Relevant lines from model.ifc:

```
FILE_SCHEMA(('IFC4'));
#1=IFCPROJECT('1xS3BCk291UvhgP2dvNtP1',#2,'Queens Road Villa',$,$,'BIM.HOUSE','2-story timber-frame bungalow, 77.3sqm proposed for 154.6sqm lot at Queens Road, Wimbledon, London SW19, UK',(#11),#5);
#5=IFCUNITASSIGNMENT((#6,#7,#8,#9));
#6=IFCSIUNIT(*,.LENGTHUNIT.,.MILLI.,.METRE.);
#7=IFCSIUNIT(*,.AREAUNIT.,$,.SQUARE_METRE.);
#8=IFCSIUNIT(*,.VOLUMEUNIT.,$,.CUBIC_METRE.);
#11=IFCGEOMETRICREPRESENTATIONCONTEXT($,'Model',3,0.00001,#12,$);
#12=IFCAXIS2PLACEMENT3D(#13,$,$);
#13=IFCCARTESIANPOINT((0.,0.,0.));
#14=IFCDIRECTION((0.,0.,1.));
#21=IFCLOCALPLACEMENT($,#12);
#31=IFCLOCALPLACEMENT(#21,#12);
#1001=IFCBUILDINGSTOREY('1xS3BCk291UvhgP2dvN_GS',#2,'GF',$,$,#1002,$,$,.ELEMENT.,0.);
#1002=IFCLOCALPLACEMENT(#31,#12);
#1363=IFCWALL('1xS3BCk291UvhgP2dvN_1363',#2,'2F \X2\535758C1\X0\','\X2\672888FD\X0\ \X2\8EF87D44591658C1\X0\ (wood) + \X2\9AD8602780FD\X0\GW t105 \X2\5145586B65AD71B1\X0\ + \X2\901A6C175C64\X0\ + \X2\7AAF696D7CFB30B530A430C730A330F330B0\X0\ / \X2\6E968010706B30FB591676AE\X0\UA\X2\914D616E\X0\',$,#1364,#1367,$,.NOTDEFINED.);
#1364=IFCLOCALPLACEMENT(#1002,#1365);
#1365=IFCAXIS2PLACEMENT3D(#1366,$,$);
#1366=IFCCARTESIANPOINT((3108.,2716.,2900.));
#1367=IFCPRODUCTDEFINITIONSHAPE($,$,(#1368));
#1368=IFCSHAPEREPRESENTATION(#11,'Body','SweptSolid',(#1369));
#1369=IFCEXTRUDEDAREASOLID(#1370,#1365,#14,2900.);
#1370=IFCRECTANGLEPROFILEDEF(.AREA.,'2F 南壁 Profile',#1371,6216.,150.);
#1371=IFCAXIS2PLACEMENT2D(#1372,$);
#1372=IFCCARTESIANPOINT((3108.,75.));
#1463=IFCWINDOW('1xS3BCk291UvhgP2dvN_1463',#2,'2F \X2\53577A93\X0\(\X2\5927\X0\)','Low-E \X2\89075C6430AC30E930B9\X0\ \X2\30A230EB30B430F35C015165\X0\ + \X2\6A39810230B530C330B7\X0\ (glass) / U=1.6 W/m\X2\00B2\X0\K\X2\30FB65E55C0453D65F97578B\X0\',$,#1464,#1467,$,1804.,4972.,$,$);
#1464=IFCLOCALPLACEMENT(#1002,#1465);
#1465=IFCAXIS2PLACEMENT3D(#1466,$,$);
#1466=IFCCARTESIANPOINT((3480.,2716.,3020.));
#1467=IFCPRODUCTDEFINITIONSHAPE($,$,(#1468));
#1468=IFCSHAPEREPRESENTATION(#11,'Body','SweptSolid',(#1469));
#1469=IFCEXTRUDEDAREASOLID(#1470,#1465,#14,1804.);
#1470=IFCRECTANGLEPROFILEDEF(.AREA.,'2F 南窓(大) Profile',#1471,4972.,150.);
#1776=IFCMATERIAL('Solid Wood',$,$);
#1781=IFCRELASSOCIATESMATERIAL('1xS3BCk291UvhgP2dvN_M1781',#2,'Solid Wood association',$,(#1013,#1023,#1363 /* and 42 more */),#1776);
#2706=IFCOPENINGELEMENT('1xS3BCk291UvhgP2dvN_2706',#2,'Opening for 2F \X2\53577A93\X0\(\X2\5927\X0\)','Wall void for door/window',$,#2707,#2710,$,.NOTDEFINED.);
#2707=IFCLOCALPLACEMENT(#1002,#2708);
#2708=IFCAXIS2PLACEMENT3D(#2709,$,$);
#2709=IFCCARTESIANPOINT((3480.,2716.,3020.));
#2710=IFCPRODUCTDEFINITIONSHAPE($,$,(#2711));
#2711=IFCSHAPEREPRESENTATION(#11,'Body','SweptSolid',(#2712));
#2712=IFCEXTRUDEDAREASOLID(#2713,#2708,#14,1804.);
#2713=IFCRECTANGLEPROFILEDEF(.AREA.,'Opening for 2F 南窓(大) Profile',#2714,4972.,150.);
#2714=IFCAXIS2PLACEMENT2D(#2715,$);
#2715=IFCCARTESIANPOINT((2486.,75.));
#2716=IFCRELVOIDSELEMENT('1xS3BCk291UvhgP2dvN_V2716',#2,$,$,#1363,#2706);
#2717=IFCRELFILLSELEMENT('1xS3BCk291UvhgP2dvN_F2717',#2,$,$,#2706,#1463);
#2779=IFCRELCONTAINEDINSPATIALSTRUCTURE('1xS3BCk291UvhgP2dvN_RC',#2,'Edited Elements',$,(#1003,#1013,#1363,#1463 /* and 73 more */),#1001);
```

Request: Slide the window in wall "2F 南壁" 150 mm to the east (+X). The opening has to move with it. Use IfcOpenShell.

```python
import ifcopenshell
import ifcopenshell.api.geometry
import ifcopenshell.util.placement
import ifcopenshell.util.unit

model = ifcopenshell.open("model.ifc")
unit_scale = ifcopenshell.util.unit.calculate_unit_scale(model)

window = model.by_id(1463)
opening = window.FillsVoids[0].RelatingOpeningElement
wall = opening.VoidsElements[0].RelatingBuildingElement

wall_matrix = ifcopenshell.util.placement.get_local_placement(wall.ObjectPlacement)
shift = wall_matrix[:3, 0] * 0.15 / unit_scale
before = ifcopenshell.util.placement.get_local_placement(window.ObjectPlacement)[:3, 3].copy()

# The window is not placed relative to its opening, so move both.
for product in (opening, window):
    matrix = ifcopenshell.util.placement.get_local_placement(product.ObjectPlacement)
    matrix[:3, 3] += shift
    ifcopenshell.api.geometry.edit_object_placement(model, product=product, matrix=matrix, is_si=False)

after = ifcopenshell.util.placement.get_local_placement(window.ObjectPlacement)[:3, 3]
print("window moved by", (after - before).round(3) + 0.0)

model.write("model_rev.ifc")
```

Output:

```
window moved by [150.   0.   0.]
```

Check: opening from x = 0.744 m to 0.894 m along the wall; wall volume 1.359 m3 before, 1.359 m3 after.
